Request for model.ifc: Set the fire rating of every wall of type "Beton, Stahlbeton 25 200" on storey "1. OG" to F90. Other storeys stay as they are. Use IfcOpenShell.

First a look at what the model holds.

```python
import ifcopenshell
import ifcopenshell.util.element

model = ifcopenshell.open("model.ifc")
print(model.schema)
storey = next(s for s in model.by_type("IfcBuildingStorey") if s.Name == "1. OG")
walls = [e for e in ifcopenshell.util.element.get_decomposition(storey) if e.is_a("IfcWall")]
seen = {}
for e in walls:
    element_type = ifcopenshell.util.element.get_type(e)
    key = (element_type.Name if element_type != e and element_type else None, ifcopenshell.util.element.get_pset(e, "Pset_WallCommon", "FireRating"))
    seen[key] = seen.get(key, 0) + 1
for (name, value), count in sorted(seen.items(), key=str):
    print(count, "x", name, "|", value)
```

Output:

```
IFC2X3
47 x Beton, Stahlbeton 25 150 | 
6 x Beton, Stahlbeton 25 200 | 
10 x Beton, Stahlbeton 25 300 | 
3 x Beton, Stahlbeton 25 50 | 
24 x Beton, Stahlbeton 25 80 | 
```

```python
import ifcopenshell
import ifcopenshell.api.pset
import ifcopenshell.util.element

model = ifcopenshell.open("model.ifc")

storey = next(s for s in model.by_type("IfcBuildingStorey") if s.Name == "1. OG")
walls = [e for e in ifcopenshell.util.element.get_decomposition(storey) if e.is_a("IfcWall")]

count = 0
for e in walls:
    element_type = ifcopenshell.util.element.get_type(e)
    if element_type in (None, e) or element_type.Name != "Beton, Stahlbeton 25 200":
        continue
    # add_pset returns the element's existing set when there is one.
    pset = ifcopenshell.api.pset.add_pset(model, product=e, name="Pset_WallCommon")
    ifcopenshell.api.pset.edit_pset(model, pset=pset, properties={"FireRating": "F90"})
    count += 1

print(count, "walls updated")

model.write("model_edited.ifc")
```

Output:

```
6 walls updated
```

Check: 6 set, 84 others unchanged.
